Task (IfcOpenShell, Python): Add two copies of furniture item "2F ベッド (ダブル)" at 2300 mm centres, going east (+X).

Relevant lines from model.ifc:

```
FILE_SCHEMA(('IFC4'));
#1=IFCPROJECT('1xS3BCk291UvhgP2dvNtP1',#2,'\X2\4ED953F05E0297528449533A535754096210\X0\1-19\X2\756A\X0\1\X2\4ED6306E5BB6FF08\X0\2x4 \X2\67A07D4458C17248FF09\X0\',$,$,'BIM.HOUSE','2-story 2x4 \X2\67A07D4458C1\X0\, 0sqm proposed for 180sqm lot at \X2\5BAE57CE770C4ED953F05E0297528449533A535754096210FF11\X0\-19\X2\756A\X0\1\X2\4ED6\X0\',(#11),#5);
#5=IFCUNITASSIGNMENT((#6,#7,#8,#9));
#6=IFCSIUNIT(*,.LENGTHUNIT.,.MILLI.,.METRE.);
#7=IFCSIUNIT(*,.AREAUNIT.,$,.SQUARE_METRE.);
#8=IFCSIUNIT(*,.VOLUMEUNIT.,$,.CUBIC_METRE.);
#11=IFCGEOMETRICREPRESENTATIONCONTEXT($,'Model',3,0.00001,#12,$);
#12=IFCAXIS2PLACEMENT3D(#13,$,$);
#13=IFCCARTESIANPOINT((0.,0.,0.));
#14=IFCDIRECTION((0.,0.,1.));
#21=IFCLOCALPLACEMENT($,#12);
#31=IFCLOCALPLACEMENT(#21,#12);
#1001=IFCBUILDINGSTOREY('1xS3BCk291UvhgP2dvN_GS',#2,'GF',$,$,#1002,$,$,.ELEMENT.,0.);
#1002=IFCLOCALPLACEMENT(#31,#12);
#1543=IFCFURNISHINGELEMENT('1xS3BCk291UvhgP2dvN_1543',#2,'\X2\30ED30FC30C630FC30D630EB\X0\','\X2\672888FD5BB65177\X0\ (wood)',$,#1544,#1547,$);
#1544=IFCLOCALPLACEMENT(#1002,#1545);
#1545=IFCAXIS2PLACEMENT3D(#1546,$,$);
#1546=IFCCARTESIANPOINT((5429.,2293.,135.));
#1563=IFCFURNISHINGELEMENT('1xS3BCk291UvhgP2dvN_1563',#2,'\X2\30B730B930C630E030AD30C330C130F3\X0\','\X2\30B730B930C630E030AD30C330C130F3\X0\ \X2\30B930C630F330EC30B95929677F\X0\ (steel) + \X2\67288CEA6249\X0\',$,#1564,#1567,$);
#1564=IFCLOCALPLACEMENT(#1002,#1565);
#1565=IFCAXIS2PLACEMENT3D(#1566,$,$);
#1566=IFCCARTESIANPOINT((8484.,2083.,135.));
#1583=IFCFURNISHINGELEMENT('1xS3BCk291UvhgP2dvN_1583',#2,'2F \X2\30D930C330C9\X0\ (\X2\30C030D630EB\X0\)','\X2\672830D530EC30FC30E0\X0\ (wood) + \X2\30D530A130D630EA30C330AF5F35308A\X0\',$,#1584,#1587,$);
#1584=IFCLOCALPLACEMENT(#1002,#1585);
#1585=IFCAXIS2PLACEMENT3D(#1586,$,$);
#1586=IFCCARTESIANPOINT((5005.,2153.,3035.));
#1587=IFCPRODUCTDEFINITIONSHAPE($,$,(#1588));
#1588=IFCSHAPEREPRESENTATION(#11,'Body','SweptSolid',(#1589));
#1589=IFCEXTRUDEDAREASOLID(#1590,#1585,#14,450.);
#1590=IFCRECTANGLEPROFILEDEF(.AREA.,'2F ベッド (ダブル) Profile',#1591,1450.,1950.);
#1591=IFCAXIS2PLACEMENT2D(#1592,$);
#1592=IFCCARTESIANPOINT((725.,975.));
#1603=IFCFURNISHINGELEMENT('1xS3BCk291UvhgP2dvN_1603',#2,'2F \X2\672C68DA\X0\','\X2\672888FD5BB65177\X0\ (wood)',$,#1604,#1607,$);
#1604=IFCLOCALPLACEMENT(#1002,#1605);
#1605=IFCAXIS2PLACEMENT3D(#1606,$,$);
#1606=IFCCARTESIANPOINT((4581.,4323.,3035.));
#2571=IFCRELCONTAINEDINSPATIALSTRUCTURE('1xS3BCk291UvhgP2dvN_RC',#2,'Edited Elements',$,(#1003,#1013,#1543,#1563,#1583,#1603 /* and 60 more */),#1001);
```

```python
import numpy as np
import ifcopenshell
import ifcopenshell.api.geometry
import ifcopenshell.api.root
import ifcopenshell.util.element
import ifcopenshell.util.placement
import ifcopenshell.util.unit

model = ifcopenshell.open("model.ifc")
unit_scale = ifcopenshell.util.unit.calculate_unit_scale(model)


def reuse_history(source, copy):
    """copy_class also copies each property set's owner history, people and application; keep the originals."""
    for rel in copy.IsDefinedBy:
        if rel.is_a("IfcRelDefinesByProperties") and (history := rel.RelatingPropertyDefinition.OwnerHistory):
            rel.RelatingPropertyDefinition.OwnerHistory = source.OwnerHistory
            ifcopenshell.util.element.remove_deep2(model, history)


source = model.by_id(1583)
base = ifcopenshell.util.placement.get_local_placement(source.ObjectPlacement)
step = np.array([1.0, 0.0, 0.0]) * 2.3 / unit_scale

for i in range(1, 3):
    copy = ifcopenshell.api.root.copy_class(model, product=source)
    copy.Representation = ifcopenshell.util.element.copy_deep(
        model, source.Representation, exclude=["IfcGeometricRepresentationContext", "IfcRepresentationMap"]
    )
    reuse_history(source, copy)
    matrix = base.copy()
    matrix[:3, 3] += i * step
    print("added at", matrix[:3, 3].round(3) + 0.0)
    ifcopenshell.api.geometry.edit_object_placement(model, product=copy, matrix=matrix, is_si=False)

model.write("model_updated.ifc")
```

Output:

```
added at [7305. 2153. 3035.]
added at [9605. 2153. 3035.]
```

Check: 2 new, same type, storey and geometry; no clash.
